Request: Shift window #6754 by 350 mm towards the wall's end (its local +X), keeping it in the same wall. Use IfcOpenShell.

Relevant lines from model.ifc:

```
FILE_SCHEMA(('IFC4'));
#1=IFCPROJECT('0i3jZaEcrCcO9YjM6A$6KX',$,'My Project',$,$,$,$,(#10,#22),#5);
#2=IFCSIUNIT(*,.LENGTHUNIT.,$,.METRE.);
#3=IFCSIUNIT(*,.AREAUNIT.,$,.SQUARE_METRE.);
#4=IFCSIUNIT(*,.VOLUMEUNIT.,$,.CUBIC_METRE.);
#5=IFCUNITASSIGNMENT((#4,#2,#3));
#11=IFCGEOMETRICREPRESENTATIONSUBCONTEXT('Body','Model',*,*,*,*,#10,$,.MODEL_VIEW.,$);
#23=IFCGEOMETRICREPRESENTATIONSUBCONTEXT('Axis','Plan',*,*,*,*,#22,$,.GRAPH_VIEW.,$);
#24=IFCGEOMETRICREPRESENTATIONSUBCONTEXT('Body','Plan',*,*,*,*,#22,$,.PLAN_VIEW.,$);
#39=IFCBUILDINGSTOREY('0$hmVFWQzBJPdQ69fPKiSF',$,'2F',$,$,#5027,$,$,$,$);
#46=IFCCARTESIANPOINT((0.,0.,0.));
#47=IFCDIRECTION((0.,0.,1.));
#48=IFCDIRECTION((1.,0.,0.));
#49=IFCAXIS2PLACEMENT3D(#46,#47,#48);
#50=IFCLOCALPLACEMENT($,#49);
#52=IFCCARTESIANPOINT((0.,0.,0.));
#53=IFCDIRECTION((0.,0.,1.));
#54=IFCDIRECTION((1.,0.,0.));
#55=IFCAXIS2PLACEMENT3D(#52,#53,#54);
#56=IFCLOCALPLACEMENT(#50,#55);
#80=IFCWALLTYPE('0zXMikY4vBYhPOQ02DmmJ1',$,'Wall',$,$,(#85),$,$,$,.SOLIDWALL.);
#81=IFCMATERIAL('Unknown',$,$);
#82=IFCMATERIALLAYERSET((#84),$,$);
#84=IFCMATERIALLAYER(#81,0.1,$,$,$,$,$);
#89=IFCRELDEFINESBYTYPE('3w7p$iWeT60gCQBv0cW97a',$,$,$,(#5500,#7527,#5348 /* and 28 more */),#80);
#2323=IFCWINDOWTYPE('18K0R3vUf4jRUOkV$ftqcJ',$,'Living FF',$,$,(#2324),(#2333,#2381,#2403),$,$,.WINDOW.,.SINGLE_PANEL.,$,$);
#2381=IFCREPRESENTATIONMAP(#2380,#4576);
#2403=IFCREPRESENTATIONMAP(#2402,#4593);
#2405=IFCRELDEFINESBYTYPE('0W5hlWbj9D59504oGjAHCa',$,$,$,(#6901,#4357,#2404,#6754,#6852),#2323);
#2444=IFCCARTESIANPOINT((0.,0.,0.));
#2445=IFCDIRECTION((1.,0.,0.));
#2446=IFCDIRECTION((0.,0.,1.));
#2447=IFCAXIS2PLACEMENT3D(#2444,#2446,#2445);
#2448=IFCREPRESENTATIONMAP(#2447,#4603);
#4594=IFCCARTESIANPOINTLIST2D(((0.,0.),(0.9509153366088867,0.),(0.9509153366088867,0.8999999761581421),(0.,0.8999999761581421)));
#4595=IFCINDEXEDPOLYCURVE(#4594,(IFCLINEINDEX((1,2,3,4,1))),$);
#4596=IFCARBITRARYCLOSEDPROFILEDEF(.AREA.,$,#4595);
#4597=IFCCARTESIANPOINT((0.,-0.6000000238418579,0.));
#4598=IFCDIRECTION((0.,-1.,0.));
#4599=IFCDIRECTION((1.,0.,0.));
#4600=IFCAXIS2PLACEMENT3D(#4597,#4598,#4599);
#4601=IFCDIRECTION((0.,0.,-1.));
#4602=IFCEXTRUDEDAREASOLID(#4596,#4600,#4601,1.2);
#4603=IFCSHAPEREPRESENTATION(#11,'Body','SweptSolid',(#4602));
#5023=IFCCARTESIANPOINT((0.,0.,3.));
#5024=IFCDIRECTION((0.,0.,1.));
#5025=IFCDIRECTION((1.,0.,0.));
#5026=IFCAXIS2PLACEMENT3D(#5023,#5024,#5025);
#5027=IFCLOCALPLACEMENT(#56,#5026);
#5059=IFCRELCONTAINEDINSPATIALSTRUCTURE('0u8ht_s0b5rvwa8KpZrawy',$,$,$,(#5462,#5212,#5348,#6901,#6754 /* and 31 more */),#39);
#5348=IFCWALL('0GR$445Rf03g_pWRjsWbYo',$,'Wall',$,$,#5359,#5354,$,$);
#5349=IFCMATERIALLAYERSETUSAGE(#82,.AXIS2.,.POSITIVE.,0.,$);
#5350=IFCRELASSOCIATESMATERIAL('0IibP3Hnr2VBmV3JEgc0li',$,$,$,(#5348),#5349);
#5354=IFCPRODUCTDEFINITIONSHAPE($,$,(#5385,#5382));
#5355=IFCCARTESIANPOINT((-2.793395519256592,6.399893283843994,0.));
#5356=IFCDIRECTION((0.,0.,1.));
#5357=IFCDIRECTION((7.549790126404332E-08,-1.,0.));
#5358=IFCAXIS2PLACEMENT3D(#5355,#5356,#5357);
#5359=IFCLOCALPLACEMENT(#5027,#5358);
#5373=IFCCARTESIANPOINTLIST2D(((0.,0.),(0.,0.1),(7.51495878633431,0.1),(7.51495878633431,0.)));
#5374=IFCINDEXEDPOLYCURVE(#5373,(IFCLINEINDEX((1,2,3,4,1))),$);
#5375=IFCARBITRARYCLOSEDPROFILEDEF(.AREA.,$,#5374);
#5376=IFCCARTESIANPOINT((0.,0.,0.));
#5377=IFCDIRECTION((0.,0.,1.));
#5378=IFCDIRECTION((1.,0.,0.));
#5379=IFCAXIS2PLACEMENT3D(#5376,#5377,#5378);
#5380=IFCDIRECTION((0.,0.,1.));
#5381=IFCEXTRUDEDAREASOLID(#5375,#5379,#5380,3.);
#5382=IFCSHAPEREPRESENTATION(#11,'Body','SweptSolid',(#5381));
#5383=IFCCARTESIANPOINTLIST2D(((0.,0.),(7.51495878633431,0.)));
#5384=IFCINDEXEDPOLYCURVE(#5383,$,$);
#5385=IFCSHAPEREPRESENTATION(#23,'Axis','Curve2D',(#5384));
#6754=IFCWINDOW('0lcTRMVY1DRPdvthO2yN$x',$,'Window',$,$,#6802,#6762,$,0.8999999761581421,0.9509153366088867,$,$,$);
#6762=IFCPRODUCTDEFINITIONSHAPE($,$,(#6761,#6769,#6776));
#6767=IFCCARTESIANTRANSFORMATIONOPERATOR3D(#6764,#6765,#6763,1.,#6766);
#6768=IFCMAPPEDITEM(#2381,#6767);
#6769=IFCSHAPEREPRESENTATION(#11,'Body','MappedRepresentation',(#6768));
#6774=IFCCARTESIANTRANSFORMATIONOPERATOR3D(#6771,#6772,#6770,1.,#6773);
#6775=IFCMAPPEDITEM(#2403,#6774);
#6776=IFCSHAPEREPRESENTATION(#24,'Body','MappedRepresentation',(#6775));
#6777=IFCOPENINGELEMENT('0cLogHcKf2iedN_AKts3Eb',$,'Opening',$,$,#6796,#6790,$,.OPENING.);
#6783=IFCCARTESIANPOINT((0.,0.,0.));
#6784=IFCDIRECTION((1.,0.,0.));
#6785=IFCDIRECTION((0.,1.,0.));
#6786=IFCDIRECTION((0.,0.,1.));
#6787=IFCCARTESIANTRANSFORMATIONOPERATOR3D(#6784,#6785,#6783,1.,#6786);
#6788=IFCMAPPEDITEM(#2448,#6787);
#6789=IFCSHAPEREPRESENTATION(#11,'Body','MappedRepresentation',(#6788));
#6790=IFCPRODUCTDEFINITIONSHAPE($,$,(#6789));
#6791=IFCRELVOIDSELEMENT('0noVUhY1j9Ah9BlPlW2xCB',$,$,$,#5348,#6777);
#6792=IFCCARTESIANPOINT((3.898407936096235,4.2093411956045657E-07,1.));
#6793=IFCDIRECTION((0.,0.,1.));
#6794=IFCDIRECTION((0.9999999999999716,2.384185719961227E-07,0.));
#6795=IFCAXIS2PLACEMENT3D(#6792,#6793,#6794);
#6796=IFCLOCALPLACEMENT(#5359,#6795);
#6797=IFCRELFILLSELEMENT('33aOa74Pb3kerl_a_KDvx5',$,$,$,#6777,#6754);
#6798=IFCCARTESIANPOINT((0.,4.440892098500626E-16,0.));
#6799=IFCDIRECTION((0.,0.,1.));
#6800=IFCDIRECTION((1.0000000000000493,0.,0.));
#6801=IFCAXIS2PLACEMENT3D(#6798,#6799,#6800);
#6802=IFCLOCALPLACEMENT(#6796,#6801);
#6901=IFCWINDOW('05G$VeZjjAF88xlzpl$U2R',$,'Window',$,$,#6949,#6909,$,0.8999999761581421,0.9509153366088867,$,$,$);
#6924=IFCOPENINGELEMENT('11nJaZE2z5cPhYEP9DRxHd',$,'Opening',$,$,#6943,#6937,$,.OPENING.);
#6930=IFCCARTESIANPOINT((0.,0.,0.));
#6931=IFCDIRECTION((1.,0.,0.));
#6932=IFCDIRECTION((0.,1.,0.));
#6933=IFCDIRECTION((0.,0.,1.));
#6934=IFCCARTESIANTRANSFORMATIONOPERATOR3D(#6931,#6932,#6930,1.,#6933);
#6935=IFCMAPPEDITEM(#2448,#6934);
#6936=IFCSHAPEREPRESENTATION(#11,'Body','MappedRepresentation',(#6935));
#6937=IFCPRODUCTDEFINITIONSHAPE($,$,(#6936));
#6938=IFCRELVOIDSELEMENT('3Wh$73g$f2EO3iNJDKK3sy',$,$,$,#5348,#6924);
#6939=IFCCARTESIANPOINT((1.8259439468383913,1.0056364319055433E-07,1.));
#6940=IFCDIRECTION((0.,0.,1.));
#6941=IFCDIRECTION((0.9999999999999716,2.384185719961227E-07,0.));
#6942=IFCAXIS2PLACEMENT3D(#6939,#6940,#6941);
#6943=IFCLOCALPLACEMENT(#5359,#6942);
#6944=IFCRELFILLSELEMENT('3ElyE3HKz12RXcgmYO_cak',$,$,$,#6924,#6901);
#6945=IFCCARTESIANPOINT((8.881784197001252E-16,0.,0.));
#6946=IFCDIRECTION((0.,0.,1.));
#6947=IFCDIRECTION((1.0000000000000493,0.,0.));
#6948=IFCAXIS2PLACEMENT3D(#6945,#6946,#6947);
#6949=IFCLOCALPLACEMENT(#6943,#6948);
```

```python
import ifcopenshell
import ifcopenshell.api.geometry
import ifcopenshell.util.placement

model = ifcopenshell.open("model.ifc")

window = model.by_id(6754)
opening = window.FillsVoids[0].RelatingOpeningElement
wall = opening.VoidsElements[0].RelatingBuildingElement

wall_matrix = ifcopenshell.util.placement.get_local_placement(wall.ObjectPlacement)
shift = wall_matrix[:3, 0] * 0.35
before = ifcopenshell.util.placement.get_local_placement(window.ObjectPlacement)[:3, 3].copy()

# The window is placed relative to its opening, so it follows when the opening moves.
matrix = ifcopenshell.util.placement.get_local_placement(opening.ObjectPlacement)
matrix[:3, 3] += shift
ifcopenshell.api.geometry.edit_object_placement(
    model, product=opening, matrix=matrix, is_si=False, should_transform_children=True
)

after = ifcopenshell.util.placement.get_local_placement(window.ObjectPlacement)[:3, 3]
print("window moved by", (after - before).round(3) + 0.0)

model.write("model_edited.ifc")
```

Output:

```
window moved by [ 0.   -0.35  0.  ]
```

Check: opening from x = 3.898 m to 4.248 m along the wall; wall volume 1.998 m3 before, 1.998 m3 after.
